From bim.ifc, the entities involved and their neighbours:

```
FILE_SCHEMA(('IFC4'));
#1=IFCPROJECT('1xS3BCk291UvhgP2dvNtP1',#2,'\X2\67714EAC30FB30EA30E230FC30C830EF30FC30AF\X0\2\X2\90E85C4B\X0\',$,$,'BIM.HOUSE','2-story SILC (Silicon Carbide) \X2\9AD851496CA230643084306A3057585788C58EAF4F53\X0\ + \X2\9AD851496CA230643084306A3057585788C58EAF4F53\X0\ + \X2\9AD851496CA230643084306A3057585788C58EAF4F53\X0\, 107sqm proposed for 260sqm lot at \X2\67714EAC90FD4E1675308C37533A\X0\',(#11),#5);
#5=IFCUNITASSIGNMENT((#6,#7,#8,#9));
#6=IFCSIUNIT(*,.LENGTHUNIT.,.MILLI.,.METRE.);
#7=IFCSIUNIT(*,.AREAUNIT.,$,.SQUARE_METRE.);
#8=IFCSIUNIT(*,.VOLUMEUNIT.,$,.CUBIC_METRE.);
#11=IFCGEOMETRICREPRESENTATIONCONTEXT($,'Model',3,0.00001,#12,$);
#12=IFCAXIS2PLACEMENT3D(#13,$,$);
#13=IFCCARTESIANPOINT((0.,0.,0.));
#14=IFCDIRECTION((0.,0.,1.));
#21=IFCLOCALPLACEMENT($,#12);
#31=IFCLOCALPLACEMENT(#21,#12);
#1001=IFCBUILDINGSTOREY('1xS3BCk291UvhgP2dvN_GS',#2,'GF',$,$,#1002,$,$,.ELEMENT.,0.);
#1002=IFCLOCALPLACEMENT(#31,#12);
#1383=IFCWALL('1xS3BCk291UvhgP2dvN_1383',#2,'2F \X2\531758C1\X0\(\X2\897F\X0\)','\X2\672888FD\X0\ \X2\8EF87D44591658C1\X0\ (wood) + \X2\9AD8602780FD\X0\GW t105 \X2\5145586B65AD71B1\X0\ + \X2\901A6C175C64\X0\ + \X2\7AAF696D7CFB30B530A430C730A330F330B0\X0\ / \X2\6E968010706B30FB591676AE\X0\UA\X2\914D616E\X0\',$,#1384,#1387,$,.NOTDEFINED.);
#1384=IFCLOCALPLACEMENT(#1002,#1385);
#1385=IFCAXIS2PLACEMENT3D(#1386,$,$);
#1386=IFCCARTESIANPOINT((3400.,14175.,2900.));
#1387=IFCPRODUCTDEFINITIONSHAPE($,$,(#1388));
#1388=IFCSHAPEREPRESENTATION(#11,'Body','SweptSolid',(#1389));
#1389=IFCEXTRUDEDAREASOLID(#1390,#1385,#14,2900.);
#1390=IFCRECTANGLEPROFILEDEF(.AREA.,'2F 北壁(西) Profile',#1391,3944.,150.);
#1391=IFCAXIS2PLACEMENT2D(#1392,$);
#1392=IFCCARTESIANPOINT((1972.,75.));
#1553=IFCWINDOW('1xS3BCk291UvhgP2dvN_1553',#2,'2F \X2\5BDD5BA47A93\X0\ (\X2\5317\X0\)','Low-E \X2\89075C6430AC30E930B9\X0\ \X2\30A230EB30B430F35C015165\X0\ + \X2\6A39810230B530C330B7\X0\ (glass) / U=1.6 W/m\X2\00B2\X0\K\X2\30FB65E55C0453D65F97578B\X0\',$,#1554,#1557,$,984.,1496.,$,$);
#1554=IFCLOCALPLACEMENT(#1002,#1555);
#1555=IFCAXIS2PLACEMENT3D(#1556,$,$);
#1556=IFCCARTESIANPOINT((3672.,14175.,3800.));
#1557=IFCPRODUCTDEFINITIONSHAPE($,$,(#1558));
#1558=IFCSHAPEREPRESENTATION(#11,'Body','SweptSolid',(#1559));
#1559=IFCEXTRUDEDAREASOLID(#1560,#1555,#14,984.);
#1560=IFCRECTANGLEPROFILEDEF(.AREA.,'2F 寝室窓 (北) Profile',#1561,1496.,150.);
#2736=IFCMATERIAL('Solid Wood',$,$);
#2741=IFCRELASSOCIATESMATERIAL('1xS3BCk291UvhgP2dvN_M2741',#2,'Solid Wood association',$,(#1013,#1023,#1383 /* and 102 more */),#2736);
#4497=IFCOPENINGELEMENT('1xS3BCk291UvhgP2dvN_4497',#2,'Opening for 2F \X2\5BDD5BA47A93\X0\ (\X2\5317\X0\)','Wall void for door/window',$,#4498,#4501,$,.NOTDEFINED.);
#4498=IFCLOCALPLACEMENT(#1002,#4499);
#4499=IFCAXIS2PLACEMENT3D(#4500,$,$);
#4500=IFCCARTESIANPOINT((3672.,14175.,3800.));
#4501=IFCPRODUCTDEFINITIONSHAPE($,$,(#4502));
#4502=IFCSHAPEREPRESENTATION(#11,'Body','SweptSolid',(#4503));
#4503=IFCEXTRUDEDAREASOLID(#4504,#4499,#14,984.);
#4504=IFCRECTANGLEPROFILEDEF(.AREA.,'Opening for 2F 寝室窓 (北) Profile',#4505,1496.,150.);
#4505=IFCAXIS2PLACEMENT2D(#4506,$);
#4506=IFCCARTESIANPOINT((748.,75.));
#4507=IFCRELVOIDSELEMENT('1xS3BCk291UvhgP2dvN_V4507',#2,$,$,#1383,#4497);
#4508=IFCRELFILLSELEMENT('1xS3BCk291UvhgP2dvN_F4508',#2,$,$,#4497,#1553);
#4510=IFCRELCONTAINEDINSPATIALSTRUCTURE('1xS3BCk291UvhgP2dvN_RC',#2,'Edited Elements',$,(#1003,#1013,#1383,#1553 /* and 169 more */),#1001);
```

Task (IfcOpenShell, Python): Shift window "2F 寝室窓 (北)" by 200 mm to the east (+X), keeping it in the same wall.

```python
import ifcopenshell
import ifcopenshell.api.geometry
import ifcopenshell.util.placement
import ifcopenshell.util.unit

model = ifcopenshell.open("bim.ifc")
unit_scale = ifcopenshell.util.unit.calculate_unit_scale(model)

window = model.by_guid("1xS3BCk291UvhgP2dvN_1553")
opening = window.FillsVoids[0].RelatingOpeningElement
wall = opening.VoidsElements[0].RelatingBuildingElement

wall_matrix = ifcopenshell.util.placement.get_local_placement(wall.ObjectPlacement)
shift = wall_matrix[:3, 0] * 0.2 / unit_scale
before = ifcopenshell.util.placement.get_local_placement(window.ObjectPlacement)[:3, 3].copy()

# The window is not placed relative to its opening, so move both.
for product in (opening, window):
    matrix = ifcopenshell.util.placement.get_local_placement(product.ObjectPlacement)
    matrix[:3, 3] += shift
    ifcopenshell.api.geometry.edit_object_placement(model, product=product, matrix=matrix, is_si=False)

after = ifcopenshell.util.placement.get_local_placement(window.ObjectPlacement)[:3, 3]
print("window moved by", (after - before).round(3) + 0.0)

model.write("bim_rev.ifc")
```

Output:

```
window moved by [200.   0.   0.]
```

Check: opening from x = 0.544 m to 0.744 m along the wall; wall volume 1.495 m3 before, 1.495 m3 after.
